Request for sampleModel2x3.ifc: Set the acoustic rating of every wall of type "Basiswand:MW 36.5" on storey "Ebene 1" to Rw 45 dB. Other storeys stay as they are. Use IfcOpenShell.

First a look at what the model holds.

```python
import ifcopenshell
import ifcopenshell.util.element

model = ifcopenshell.open("sampleModel2x3.ifc")
print(model.schema)
storey = next(s for s in model.by_type("IfcBuildingStorey") if s.Name == "Ebene 1")
walls = [e for e in ifcopenshell.util.element.get_decomposition(storey) if e.is_a("IfcWall")]
seen = {}
for e in walls:
    element_type = ifcopenshell.util.element.get_type(e)
    key = (element_type.Name if element_type != e and element_type else None, ifcopenshell.util.element.get_pset(e, "Pset_WallCommon", "AcousticRating"))
    seen[key] = seen.get(key, 0) + 1
for (name, value), count in sorted(seen.items(), key=str):
    print(count, "x", name, "|", value)
```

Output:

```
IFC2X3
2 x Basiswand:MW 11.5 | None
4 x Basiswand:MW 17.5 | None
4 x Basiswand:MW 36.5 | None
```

```python
import ifcopenshell
import ifcopenshell.api.pset
import ifcopenshell.util.element

model = ifcopenshell.open("sampleModel2x3.ifc")

storey = next(s for s in model.by_type("IfcBuildingStorey") if s.Name == "Ebene 1")
walls = [e for e in ifcopenshell.util.element.get_decomposition(storey) if e.is_a("IfcWall")]

count = 0
for e in walls:
    element_type = ifcopenshell.util.element.get_type(e)
    if element_type in (None, e) or element_type.Name != "Basiswand:MW 36.5":
        continue
    # add_pset returns the element's existing set when there is one.
    pset = ifcopenshell.api.pset.add_pset(model, product=e, name="Pset_WallCommon")
    ifcopenshell.api.pset.edit_pset(model, pset=pset, properties={"AcousticRating": "Rw 45 dB"})
    count += 1

print(count, "walls updated")

model.write("sampleModel2x3-out.ifc")
```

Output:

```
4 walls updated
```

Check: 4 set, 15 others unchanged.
